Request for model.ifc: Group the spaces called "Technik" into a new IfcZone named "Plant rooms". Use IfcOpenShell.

First a look at what the model holds.

```python
import ifcopenshell

model = ifcopenshell.open("model.ifc")
print(model.schema)
seen = {}
for space in model.by_type("IfcSpace"):
    seen[space.LongName] = seen.get(space.LongName, 0) + 1
for name, count in sorted(seen.items(), key=str):
    print(count, "x", name)
print("zones:", [z.Name for z in model.by_type("IfcZone")][:20])
```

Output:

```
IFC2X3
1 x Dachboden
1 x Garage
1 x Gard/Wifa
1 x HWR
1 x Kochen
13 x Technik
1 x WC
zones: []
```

```python
import ifcopenshell
import ifcopenshell.api.group
import ifcopenshell.api.root

model = ifcopenshell.open("model.ifc")

names = {"Technik"}
spaces = [s for s in model.by_type("IfcSpace") if s.LongName in names]

zone = ifcopenshell.api.root.create_entity(model, ifc_class="IfcZone", name="Plant rooms")
ifcopenshell.api.group.assign_group(model, products=spaces, group=zone)
print(len(spaces), "spaces in", zone.Name)

model.write("model_rev.ifc")
```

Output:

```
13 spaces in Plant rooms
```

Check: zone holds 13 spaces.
